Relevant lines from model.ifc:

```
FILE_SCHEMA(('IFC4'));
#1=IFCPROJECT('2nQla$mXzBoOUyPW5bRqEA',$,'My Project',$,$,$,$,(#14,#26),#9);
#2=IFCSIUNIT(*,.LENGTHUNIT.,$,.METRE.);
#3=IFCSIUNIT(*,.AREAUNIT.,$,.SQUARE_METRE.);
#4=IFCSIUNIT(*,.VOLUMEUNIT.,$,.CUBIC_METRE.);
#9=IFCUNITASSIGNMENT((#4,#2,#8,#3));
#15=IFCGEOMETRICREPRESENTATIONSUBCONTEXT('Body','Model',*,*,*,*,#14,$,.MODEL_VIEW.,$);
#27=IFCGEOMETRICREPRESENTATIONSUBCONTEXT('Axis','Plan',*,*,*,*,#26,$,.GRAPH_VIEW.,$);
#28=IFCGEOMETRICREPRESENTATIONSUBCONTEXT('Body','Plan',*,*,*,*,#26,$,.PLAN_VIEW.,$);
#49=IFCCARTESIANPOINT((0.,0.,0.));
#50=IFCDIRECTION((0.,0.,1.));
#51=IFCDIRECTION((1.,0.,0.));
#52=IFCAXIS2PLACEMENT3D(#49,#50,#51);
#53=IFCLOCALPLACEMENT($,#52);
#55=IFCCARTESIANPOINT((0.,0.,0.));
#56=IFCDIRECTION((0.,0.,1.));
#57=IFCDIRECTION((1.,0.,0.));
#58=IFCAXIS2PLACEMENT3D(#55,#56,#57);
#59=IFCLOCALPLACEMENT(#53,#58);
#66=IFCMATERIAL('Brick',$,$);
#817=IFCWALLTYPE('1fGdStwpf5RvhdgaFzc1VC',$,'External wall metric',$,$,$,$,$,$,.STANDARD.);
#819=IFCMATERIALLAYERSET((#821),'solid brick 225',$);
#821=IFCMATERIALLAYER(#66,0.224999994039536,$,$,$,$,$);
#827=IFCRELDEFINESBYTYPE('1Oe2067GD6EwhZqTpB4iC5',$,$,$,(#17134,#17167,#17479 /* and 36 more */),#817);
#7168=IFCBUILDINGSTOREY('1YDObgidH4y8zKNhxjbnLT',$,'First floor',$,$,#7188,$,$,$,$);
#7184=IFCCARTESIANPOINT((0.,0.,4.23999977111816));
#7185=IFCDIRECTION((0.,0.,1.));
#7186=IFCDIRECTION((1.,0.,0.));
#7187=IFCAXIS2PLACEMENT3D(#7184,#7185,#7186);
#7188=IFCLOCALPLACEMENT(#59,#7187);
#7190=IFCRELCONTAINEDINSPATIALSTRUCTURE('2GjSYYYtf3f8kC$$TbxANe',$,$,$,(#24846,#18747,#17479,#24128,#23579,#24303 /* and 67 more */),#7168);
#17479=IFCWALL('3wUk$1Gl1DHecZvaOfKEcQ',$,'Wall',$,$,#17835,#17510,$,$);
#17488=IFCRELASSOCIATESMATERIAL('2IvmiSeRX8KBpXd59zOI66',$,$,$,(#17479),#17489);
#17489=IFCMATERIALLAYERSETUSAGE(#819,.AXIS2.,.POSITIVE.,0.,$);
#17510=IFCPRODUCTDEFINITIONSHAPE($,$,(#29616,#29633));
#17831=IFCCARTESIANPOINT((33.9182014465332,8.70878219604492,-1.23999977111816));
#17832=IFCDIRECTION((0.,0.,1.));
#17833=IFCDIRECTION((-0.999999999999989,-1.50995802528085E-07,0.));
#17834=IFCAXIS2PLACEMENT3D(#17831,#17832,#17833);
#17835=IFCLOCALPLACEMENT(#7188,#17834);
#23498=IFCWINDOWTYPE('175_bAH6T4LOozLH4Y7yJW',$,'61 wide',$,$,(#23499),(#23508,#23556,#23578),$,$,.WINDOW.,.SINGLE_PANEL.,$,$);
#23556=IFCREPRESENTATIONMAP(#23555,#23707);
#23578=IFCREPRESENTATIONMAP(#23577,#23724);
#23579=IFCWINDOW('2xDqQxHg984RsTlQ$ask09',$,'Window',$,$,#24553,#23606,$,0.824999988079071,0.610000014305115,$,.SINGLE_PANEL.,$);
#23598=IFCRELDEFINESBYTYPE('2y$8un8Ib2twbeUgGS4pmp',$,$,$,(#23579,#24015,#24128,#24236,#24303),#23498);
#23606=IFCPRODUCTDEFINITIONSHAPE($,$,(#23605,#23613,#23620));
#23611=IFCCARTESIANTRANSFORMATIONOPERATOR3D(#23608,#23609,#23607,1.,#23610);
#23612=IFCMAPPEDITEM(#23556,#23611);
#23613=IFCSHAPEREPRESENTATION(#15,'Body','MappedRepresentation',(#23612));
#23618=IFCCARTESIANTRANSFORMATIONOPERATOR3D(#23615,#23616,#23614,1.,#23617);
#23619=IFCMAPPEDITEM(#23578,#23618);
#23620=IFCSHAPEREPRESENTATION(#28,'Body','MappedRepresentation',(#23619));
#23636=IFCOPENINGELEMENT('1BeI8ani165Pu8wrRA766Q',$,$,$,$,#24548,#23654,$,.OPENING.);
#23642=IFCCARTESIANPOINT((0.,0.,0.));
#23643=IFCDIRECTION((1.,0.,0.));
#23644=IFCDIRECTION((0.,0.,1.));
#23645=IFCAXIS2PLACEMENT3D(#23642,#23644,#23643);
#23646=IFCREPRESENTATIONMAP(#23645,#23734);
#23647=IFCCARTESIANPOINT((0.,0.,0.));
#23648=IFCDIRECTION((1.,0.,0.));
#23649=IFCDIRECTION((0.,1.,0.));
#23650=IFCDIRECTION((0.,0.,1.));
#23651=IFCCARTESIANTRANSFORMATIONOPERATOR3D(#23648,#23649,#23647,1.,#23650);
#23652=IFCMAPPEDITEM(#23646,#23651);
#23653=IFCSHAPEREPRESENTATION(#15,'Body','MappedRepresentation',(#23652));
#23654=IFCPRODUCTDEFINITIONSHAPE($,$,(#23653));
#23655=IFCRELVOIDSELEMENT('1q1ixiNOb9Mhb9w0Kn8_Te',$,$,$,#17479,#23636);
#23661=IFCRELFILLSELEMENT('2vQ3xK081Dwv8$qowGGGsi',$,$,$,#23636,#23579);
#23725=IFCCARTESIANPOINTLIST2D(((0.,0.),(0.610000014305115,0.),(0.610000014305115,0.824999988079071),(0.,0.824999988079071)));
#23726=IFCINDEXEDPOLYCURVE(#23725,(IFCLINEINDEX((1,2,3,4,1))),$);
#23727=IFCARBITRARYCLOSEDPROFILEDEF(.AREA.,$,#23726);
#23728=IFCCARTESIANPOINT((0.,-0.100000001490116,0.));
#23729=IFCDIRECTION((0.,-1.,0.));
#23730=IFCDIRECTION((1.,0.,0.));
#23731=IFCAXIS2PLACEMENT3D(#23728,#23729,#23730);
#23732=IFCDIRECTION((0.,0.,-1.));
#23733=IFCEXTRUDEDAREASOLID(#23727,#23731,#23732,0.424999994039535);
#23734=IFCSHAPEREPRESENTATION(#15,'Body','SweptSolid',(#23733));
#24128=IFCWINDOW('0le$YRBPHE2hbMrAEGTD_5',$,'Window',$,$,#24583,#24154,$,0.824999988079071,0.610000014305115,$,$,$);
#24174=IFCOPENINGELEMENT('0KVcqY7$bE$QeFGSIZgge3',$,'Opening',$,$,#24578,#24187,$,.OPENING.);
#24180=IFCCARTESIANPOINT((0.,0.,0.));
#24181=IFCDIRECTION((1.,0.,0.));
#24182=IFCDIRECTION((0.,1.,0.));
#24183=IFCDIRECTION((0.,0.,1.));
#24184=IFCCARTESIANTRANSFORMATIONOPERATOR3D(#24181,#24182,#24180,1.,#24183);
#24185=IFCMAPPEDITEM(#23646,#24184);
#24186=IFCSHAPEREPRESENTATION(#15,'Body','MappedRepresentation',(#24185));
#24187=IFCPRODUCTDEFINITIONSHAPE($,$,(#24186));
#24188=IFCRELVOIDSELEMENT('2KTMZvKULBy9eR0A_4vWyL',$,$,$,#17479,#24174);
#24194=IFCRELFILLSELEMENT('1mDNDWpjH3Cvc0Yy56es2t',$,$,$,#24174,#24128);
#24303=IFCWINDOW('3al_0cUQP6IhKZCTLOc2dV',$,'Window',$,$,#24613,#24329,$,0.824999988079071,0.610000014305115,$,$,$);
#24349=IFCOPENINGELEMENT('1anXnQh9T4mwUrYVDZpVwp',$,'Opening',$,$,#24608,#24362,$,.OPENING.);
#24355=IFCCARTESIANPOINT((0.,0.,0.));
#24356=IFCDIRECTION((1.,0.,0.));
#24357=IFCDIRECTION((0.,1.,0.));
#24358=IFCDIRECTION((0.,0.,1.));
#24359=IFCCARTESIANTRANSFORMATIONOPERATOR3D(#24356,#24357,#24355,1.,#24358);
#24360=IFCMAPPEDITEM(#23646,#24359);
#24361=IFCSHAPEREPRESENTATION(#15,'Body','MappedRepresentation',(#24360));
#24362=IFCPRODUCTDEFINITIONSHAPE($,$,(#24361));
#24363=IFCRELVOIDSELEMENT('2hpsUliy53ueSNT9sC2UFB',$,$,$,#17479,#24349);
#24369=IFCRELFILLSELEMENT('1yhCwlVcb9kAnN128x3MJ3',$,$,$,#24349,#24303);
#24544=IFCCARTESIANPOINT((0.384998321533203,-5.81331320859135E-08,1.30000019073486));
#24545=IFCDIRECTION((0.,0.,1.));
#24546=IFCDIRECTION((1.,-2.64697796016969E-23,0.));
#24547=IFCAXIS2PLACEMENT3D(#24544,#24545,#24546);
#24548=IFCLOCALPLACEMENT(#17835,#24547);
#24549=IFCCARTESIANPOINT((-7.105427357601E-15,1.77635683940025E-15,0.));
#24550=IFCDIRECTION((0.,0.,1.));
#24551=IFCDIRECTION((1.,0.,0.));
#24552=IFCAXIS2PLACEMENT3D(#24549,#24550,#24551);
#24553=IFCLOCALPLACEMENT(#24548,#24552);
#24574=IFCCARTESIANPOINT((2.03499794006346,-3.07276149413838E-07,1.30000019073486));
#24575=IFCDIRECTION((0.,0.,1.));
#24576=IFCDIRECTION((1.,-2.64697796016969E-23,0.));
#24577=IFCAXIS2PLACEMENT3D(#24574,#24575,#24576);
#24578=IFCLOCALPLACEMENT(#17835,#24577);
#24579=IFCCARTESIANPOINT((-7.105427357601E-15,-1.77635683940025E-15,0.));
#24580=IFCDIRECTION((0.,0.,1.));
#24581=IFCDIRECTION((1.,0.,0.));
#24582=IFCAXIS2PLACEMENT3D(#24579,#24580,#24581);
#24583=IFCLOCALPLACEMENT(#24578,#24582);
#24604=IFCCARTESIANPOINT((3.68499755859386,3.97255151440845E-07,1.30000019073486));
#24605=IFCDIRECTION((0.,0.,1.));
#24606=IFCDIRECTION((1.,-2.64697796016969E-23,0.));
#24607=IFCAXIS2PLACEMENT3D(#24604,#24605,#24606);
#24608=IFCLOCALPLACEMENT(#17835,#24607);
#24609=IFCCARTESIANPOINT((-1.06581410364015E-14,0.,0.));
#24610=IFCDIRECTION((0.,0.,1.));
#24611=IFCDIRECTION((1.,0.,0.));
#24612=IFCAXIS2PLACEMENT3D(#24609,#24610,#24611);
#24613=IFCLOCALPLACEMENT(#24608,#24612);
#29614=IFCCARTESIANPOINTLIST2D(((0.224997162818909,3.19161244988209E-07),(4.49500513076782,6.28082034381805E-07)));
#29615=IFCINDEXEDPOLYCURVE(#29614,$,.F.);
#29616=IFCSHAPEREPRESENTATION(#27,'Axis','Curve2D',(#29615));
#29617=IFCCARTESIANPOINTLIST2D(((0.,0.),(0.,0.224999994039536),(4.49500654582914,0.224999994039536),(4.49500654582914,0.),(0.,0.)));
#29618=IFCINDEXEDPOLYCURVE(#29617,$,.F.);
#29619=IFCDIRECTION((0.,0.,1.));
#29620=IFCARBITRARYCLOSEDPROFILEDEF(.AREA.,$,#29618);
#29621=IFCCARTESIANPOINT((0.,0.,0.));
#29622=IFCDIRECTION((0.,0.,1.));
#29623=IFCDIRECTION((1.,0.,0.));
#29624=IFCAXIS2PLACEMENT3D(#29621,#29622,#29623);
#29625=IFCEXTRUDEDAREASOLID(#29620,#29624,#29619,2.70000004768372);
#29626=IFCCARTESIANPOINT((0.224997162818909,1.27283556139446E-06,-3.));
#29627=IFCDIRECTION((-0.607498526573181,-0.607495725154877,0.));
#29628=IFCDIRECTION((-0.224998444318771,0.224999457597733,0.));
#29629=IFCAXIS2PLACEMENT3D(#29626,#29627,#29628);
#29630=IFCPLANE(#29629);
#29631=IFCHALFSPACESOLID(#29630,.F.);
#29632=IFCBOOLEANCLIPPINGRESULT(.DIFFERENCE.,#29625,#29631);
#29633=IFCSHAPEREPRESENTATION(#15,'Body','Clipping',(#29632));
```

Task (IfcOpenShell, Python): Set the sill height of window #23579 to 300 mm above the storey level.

```python
import numpy as np
import ifcopenshell
import ifcopenshell.api.geometry
import ifcopenshell.geom
import ifcopenshell.util.element
import ifcopenshell.util.placement
import ifcopenshell.util.shape
import ifcopenshell.util.unit

model = ifcopenshell.open("model.ifc")
unit_scale = ifcopenshell.util.unit.calculate_unit_scale(model)

window = model.by_guid("2xDqQxHg984RsTlQ$ask09")
opening = window.FillsVoids[0].RelatingOpeningElement
storey = ifcopenshell.util.element.get_container(window, ifc_class="IfcBuildingStorey")
level = ifcopenshell.util.placement.get_local_placement(storey.ObjectPlacement)[2, 3]

# The opening's origin need not be at the sill, so measure its lowest point.
shape = ifcopenshell.geom.create_shape(ifcopenshell.geom.settings(), opening)
bottom = ifcopenshell.util.shape.get_shape_bottom_elevation(shape, shape.geometry) / unit_scale
dz = level + 0.3 - bottom

shift = np.array([0.0, 0.0, dz])
# The window is placed relative to its opening, so it follows when the opening moves.
matrix = ifcopenshell.util.placement.get_local_placement(opening.ObjectPlacement)
matrix[:3, 3] += shift
ifcopenshell.api.geometry.edit_object_placement(
    model, product=opening, matrix=matrix, is_si=False, should_transform_children=True
)

print(f"moved by {dz * unit_scale:+.3f} m")

model.write("model-out.ifc")
```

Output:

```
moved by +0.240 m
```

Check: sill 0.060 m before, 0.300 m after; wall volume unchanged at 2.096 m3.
